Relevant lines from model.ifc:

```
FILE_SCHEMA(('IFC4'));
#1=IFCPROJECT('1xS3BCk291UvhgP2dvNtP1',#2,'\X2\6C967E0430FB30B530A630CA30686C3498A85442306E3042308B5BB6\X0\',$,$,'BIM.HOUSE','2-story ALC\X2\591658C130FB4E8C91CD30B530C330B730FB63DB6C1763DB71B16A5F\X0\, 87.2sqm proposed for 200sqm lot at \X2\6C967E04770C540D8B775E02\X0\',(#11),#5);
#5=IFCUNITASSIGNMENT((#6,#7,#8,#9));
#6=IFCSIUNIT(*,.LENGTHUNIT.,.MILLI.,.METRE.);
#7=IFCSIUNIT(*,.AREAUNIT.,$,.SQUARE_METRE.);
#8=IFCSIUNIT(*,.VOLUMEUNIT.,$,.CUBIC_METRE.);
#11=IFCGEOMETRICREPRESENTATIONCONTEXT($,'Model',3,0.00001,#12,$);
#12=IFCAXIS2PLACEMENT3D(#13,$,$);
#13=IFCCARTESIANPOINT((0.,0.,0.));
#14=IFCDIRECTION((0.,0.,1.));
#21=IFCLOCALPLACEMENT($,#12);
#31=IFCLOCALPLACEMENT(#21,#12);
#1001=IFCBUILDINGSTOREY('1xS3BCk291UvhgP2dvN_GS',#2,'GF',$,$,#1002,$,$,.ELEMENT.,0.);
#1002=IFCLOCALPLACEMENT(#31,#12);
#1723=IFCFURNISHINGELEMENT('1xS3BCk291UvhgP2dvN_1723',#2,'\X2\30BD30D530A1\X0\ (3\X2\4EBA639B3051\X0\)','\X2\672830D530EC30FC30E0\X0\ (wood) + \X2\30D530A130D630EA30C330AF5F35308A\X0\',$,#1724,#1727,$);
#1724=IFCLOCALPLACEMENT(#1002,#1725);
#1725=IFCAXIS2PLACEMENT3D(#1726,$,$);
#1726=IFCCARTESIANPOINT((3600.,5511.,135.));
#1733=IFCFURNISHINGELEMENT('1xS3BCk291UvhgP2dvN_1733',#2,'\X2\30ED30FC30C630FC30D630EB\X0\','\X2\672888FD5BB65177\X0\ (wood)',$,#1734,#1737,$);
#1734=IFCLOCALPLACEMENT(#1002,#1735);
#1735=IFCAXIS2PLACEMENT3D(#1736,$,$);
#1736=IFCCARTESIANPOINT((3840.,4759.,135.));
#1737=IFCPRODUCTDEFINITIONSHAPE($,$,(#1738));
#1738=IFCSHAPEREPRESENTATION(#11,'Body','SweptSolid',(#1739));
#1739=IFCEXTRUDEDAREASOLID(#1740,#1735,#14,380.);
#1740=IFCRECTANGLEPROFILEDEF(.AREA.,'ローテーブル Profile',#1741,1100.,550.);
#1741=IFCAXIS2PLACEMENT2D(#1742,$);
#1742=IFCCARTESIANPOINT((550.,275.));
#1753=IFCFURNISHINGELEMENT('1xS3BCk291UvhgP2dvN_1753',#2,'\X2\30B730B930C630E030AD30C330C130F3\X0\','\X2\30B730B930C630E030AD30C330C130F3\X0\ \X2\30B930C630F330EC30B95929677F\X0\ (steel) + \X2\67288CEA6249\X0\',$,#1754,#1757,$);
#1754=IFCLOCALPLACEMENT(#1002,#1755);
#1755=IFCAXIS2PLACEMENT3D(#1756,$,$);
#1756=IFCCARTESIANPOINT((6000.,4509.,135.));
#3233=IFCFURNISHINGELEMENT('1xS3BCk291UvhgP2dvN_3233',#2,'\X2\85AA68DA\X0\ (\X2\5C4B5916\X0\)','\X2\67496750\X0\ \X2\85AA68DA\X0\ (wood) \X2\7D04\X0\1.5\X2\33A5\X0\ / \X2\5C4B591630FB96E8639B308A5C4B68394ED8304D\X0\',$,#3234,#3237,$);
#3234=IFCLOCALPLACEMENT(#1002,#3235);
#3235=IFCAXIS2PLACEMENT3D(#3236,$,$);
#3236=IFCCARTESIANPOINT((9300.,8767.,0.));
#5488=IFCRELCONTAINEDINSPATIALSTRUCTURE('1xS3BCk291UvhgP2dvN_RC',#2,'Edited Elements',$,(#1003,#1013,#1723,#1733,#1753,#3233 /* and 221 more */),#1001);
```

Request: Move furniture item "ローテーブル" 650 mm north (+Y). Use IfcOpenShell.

```python
import ifcopenshell
import ifcopenshell.api.geometry
import ifcopenshell.util.placement

model = ifcopenshell.open("model.ifc")

item = model.by_guid("1xS3BCk291UvhgP2dvN_1733")
matrix = ifcopenshell.util.placement.get_local_placement(item.ObjectPlacement)
matrix[1, 3] += 650.0
ifcopenshell.api.geometry.edit_object_placement(model, product=item, matrix=matrix, is_si=False)

print(ifcopenshell.util.placement.get_local_placement(item.ObjectPlacement).round(3) + 0.0)

model.write("model-out.ifc")
```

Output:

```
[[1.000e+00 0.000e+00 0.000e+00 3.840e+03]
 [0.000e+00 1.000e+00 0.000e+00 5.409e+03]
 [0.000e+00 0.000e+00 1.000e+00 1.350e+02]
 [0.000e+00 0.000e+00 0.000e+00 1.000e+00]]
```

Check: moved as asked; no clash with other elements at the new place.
